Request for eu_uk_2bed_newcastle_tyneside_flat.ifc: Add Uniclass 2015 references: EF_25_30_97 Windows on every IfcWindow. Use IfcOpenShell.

First a look at what the model holds.

```python
import ifcopenshell

model = ifcopenshell.open("eu_uk_2bed_newcastle_tyneside_flat.ifc")
print(model.schema)
print("classifications:", [c.Name for c in model.by_type("IfcClassification")])
for ifc_class in ("IfcDoor", "IfcRoof", "IfcStair", "IfcWall", "IfcWindow"):
    print(ifc_class, len(model.by_type(ifc_class)))
```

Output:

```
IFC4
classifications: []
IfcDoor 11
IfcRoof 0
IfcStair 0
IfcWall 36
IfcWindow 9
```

```python
import ifcopenshell
import ifcopenshell.api.classification

model = ifcopenshell.open("eu_uk_2bed_newcastle_tyneside_flat.ifc")

system = ifcopenshell.api.classification.add_classification(model, classification="Uniclass 2015")

codes = {
    "IfcWindow": ("EF_25_30_97", "Windows"),
}
for ifc_class, (code, name) in codes.items():
    products = model.by_type(ifc_class)
    ifcopenshell.api.classification.add_reference(
        model, products=products, classification=system, identification=code, name=name
    )
    print(code, len(products))

model.write("eu_uk_2bed_newcastle_tyneside_flat_edited.ifc")
```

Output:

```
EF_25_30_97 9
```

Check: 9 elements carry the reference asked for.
